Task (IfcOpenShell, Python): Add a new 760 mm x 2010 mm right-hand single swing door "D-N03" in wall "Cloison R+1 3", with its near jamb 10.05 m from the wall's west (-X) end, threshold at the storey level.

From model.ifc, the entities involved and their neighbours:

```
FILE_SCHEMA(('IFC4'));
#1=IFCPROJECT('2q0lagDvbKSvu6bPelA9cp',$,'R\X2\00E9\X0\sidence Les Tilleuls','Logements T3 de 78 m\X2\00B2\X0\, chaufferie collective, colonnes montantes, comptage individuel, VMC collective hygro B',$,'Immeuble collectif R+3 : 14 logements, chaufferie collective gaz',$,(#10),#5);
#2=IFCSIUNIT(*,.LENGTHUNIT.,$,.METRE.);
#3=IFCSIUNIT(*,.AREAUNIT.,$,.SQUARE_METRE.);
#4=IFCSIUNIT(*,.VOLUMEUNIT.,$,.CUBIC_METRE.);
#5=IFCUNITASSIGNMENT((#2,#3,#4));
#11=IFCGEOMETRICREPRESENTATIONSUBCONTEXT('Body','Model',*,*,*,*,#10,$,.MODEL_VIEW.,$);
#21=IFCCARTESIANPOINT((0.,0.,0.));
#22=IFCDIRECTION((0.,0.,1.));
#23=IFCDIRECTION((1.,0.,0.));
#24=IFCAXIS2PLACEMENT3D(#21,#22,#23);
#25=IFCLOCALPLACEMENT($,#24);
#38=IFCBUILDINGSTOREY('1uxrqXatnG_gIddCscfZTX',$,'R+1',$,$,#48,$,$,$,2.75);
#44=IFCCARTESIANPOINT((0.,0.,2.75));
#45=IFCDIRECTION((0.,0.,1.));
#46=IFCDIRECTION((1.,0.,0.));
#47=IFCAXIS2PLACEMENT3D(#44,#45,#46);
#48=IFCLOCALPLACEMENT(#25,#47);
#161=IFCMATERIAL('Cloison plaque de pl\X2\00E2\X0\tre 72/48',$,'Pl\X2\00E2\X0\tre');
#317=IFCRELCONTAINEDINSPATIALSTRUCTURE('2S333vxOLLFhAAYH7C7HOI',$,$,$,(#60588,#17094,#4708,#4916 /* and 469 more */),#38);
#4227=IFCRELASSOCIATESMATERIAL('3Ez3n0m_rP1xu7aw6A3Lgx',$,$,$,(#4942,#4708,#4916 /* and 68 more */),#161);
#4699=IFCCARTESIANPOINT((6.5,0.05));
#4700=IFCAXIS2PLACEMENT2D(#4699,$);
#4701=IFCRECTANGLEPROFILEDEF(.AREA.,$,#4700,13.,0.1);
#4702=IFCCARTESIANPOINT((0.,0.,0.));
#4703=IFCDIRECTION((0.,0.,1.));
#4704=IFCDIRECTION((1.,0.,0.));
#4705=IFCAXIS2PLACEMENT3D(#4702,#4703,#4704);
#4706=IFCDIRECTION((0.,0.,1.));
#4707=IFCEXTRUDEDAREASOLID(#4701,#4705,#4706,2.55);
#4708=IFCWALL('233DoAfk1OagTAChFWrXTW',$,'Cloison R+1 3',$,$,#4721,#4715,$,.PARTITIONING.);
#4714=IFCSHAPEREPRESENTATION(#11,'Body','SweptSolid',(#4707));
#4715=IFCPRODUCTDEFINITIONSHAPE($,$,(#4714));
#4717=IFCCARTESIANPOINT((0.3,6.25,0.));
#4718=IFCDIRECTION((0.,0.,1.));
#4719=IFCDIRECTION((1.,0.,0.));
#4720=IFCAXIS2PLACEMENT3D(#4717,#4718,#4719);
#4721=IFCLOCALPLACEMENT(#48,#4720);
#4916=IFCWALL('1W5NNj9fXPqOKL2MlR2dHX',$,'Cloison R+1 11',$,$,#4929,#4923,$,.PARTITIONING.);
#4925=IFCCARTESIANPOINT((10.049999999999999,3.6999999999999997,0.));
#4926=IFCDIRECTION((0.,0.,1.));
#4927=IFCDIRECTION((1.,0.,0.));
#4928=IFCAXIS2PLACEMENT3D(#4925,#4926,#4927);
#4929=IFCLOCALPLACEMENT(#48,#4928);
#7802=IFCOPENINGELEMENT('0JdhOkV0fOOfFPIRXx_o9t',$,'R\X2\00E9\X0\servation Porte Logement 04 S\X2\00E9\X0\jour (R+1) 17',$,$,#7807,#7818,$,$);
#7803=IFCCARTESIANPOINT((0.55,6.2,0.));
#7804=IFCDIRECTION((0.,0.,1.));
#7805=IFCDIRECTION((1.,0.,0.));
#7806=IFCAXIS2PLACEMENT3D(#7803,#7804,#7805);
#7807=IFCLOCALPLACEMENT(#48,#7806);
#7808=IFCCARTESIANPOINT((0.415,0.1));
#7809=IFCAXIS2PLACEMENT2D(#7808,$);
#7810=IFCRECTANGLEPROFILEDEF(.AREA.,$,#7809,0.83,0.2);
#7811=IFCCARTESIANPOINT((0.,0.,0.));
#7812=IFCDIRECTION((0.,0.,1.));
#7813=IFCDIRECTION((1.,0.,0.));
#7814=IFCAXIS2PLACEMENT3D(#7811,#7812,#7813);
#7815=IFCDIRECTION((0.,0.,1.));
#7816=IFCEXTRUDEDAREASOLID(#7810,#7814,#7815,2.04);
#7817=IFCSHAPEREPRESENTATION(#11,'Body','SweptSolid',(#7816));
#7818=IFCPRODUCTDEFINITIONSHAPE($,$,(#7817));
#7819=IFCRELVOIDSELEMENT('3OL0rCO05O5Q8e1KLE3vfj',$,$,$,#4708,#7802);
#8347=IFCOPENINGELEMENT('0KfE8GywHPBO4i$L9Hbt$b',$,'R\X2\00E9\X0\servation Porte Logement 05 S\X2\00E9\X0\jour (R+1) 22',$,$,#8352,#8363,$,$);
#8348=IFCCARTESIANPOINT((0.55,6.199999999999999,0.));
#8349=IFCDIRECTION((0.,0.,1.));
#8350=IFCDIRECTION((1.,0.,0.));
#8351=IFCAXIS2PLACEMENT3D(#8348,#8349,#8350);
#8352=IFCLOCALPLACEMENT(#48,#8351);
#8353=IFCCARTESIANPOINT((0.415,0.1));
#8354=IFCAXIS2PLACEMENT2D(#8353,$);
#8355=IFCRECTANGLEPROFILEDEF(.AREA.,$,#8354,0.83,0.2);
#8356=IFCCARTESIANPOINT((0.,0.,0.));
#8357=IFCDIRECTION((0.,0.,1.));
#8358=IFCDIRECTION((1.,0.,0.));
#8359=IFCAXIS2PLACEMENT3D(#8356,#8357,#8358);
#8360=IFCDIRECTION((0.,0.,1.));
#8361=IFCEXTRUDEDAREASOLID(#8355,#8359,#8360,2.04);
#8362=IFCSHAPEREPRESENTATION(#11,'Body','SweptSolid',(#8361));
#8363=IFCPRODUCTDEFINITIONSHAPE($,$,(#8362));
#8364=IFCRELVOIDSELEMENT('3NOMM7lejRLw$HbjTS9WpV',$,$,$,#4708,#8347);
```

```python
import numpy as np
import ifcopenshell
import ifcopenshell.api.feature
import ifcopenshell.api.geometry
import ifcopenshell.api.root
import ifcopenshell.api.spatial
import ifcopenshell.geom
import ifcopenshell.util.element
import ifcopenshell.util.placement
import ifcopenshell.util.representation
import ifcopenshell.util.shape
import ifcopenshell.util.unit

model = ifcopenshell.open("model.ifc")
unit_scale = ifcopenshell.util.unit.calculate_unit_scale(model)
settings = ifcopenshell.geom.settings()


def volume(element):
    """Net volume in cubic metres, openings subtracted."""
    shape = ifcopenshell.geom.create_shape(settings, element)
    return ifcopenshell.util.shape.get_volume(shape.geometry)


wall = model.by_guid("233DoAfk1OagTAChFWrXTW")
storey = ifcopenshell.util.element.get_container(wall, ifc_class="IfcBuildingStorey")
context = ifcopenshell.util.representation.get_context(model, "Model", "Body", "MODEL_VIEW")
before = volume(wall)

width, height, from_end, sill = 0.76, 2.01, 10.05, 0.0  # metres

# The wall runs along its own X axis, and the end named is its -X end.
wall_shape = ifcopenshell.geom.create_shape(settings, wall)
x, y, z = ifcopenshell.util.shape.get_vertices(wall_shape.geometry).T
start = x.min() + from_end
face, thickness = float(y.min()), float(y.max() - y.min())
wall_matrix = ifcopenshell.util.placement.get_local_placement(wall.ObjectPlacement)
level = ifcopenshell.util.placement.get_local_placement(storey.ObjectPlacement)[2, 3]


def in_wall(x, y):
    """Placement at x, y metres in the wall's axes, at sill height."""
    matrix = wall_matrix.copy()
    matrix[:, 3] = wall_matrix @ np.array([x / unit_scale, y / unit_scale, 0.0, 1.0])
    matrix[2, 3] = level + sill / unit_scale
    return matrix


# Opening: a box that overshoots both wall faces by 50 mm.
opening = ifcopenshell.api.root.create_entity(model, ifc_class="IfcOpeningElement", predefined_type="OPENING")
box = ifcopenshell.api.geometry.add_wall_representation(
    model, context=context, length=width, height=height, thickness=thickness + 0.1
)
ifcopenshell.api.geometry.assign_representation(model, product=opening, representation=box)
ifcopenshell.api.geometry.edit_object_placement(model, product=opening, matrix=in_wall(start, face - 0.05), is_si=False)
ifcopenshell.api.feature.add_feature(model, feature=opening, element=wall)

door = ifcopenshell.api.root.create_entity(model, ifc_class="IfcDoor", name="D-N03", predefined_type="DOOR")
door.OverallWidth, door.OverallHeight = width / unit_scale, height / unit_scale
door.OperationType = "SINGLE_SWING_RIGHT"
body = ifcopenshell.api.geometry.add_door_representation(
    model,
    context=context,
    overall_width=door.OverallWidth,
    overall_height=door.OverallHeight,
    operation_type="SINGLE_SWING_RIGHT",
    lining_properties={"LiningDepth": thickness / unit_scale, "ThresholdDepth": thickness / unit_scale},
)
ifcopenshell.api.geometry.assign_representation(model, product=door, representation=body)
ifcopenshell.api.spatial.assign_container(model, products=[door], relating_structure=storey)
ifcopenshell.api.feature.add_filling(model, opening=opening, element=door)

# The lining spans the wall, so the door starts at the wall face.
ifcopenshell.api.geometry.edit_object_placement(model, product=door, matrix=in_wall(start, face), is_si=False)

after = volume(wall)

print(f"wall volume {before:.3f} -> {after:.3f} m3")

model.write("model_rev.ifc")
```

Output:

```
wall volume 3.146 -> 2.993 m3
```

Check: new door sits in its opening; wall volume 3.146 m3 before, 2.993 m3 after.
